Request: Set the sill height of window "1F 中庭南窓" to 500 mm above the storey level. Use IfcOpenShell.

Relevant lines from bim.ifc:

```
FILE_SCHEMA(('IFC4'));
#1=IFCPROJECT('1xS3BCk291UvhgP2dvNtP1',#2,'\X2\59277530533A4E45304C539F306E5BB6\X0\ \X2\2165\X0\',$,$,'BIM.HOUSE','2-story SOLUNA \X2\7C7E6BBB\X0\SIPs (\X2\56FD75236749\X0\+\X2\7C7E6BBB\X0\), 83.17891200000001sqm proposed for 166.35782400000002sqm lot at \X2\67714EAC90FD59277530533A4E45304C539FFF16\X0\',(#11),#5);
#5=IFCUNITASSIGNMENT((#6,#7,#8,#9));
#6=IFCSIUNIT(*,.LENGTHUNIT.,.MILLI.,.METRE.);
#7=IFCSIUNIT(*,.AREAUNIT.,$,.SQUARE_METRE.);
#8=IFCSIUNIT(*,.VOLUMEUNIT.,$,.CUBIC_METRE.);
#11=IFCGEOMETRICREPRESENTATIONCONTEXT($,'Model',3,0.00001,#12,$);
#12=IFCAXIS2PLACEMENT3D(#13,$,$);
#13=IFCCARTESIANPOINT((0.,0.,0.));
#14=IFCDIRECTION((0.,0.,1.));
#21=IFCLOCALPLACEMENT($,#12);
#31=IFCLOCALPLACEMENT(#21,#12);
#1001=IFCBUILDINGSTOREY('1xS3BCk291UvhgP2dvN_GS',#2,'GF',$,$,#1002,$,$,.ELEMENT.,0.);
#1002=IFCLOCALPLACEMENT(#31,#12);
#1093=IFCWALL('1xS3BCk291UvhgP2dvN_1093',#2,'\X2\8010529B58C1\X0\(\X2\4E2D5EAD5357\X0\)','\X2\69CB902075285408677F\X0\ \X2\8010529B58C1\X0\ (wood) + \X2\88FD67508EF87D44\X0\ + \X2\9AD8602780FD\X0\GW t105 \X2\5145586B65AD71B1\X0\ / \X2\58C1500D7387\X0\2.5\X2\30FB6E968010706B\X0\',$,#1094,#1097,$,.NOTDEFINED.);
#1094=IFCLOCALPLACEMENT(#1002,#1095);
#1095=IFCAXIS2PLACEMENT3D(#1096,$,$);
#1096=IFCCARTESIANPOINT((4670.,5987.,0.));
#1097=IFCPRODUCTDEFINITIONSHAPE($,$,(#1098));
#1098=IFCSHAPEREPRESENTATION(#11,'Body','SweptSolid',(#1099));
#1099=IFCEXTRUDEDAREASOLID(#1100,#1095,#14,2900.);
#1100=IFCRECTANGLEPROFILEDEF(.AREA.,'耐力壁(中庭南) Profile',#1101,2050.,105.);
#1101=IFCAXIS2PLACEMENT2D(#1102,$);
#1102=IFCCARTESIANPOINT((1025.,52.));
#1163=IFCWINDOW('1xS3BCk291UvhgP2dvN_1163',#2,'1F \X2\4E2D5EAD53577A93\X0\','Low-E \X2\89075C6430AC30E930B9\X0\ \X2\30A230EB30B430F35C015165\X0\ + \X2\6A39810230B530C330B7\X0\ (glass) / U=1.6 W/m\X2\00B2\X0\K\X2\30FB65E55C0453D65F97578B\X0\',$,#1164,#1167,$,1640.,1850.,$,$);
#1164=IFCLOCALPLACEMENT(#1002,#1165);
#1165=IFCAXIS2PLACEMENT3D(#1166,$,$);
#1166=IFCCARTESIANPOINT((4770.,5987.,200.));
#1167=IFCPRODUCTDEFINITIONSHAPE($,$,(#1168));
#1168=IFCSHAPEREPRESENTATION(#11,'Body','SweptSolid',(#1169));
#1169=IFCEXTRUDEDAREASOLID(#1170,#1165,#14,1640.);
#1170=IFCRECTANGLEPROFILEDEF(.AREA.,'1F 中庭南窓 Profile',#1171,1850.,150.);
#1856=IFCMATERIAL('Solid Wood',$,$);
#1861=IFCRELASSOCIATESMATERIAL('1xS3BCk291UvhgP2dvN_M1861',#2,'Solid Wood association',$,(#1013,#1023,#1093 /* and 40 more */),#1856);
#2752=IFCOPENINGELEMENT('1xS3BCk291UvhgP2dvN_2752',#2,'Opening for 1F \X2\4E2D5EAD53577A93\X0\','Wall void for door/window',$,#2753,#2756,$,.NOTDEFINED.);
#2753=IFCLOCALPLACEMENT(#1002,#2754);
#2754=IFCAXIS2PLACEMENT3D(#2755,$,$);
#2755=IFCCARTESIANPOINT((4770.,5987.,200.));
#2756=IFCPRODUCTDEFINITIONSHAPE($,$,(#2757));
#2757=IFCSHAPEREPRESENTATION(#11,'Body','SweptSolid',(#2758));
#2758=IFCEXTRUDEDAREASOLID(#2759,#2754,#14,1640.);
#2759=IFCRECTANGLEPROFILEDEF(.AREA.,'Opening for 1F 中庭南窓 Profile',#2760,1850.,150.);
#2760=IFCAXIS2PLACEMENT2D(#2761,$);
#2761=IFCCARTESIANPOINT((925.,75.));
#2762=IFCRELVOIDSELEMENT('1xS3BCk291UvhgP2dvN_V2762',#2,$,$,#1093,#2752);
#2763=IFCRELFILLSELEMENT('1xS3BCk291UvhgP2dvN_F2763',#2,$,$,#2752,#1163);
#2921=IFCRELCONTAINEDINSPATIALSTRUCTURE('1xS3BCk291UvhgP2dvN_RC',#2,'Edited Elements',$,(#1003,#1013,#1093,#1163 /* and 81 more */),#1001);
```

```python
import numpy as np
import ifcopenshell
import ifcopenshell.api.geometry
import ifcopenshell.geom
import ifcopenshell.util.element
import ifcopenshell.util.placement
import ifcopenshell.util.shape
import ifcopenshell.util.unit

model = ifcopenshell.open("bim.ifc")
unit_scale = ifcopenshell.util.unit.calculate_unit_scale(model)

window = model.by_guid("1xS3BCk291UvhgP2dvN_1163")
opening = window.FillsVoids[0].RelatingOpeningElement
storey = ifcopenshell.util.element.get_container(window, ifc_class="IfcBuildingStorey")
level = ifcopenshell.util.placement.get_local_placement(storey.ObjectPlacement)[2, 3]

# The opening's origin need not be at the sill, so measure its lowest point.
shape = ifcopenshell.geom.create_shape(ifcopenshell.geom.settings(), opening)
bottom = ifcopenshell.util.shape.get_shape_bottom_elevation(shape, shape.geometry) / unit_scale
dz = level + 0.5 / unit_scale - bottom

shift = np.array([0.0, 0.0, dz])
# The window is not placed relative to its opening, so move both.
for product in (opening, window):
    matrix = ifcopenshell.util.placement.get_local_placement(product.ObjectPlacement)
    matrix[:3, 3] += shift
    ifcopenshell.api.geometry.edit_object_placement(model, product=product, matrix=matrix, is_si=False)

print(f"moved by {dz * unit_scale:+.3f} m")

model.write("bim_v2.ifc")
```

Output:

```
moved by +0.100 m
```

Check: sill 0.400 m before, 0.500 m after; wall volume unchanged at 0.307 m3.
